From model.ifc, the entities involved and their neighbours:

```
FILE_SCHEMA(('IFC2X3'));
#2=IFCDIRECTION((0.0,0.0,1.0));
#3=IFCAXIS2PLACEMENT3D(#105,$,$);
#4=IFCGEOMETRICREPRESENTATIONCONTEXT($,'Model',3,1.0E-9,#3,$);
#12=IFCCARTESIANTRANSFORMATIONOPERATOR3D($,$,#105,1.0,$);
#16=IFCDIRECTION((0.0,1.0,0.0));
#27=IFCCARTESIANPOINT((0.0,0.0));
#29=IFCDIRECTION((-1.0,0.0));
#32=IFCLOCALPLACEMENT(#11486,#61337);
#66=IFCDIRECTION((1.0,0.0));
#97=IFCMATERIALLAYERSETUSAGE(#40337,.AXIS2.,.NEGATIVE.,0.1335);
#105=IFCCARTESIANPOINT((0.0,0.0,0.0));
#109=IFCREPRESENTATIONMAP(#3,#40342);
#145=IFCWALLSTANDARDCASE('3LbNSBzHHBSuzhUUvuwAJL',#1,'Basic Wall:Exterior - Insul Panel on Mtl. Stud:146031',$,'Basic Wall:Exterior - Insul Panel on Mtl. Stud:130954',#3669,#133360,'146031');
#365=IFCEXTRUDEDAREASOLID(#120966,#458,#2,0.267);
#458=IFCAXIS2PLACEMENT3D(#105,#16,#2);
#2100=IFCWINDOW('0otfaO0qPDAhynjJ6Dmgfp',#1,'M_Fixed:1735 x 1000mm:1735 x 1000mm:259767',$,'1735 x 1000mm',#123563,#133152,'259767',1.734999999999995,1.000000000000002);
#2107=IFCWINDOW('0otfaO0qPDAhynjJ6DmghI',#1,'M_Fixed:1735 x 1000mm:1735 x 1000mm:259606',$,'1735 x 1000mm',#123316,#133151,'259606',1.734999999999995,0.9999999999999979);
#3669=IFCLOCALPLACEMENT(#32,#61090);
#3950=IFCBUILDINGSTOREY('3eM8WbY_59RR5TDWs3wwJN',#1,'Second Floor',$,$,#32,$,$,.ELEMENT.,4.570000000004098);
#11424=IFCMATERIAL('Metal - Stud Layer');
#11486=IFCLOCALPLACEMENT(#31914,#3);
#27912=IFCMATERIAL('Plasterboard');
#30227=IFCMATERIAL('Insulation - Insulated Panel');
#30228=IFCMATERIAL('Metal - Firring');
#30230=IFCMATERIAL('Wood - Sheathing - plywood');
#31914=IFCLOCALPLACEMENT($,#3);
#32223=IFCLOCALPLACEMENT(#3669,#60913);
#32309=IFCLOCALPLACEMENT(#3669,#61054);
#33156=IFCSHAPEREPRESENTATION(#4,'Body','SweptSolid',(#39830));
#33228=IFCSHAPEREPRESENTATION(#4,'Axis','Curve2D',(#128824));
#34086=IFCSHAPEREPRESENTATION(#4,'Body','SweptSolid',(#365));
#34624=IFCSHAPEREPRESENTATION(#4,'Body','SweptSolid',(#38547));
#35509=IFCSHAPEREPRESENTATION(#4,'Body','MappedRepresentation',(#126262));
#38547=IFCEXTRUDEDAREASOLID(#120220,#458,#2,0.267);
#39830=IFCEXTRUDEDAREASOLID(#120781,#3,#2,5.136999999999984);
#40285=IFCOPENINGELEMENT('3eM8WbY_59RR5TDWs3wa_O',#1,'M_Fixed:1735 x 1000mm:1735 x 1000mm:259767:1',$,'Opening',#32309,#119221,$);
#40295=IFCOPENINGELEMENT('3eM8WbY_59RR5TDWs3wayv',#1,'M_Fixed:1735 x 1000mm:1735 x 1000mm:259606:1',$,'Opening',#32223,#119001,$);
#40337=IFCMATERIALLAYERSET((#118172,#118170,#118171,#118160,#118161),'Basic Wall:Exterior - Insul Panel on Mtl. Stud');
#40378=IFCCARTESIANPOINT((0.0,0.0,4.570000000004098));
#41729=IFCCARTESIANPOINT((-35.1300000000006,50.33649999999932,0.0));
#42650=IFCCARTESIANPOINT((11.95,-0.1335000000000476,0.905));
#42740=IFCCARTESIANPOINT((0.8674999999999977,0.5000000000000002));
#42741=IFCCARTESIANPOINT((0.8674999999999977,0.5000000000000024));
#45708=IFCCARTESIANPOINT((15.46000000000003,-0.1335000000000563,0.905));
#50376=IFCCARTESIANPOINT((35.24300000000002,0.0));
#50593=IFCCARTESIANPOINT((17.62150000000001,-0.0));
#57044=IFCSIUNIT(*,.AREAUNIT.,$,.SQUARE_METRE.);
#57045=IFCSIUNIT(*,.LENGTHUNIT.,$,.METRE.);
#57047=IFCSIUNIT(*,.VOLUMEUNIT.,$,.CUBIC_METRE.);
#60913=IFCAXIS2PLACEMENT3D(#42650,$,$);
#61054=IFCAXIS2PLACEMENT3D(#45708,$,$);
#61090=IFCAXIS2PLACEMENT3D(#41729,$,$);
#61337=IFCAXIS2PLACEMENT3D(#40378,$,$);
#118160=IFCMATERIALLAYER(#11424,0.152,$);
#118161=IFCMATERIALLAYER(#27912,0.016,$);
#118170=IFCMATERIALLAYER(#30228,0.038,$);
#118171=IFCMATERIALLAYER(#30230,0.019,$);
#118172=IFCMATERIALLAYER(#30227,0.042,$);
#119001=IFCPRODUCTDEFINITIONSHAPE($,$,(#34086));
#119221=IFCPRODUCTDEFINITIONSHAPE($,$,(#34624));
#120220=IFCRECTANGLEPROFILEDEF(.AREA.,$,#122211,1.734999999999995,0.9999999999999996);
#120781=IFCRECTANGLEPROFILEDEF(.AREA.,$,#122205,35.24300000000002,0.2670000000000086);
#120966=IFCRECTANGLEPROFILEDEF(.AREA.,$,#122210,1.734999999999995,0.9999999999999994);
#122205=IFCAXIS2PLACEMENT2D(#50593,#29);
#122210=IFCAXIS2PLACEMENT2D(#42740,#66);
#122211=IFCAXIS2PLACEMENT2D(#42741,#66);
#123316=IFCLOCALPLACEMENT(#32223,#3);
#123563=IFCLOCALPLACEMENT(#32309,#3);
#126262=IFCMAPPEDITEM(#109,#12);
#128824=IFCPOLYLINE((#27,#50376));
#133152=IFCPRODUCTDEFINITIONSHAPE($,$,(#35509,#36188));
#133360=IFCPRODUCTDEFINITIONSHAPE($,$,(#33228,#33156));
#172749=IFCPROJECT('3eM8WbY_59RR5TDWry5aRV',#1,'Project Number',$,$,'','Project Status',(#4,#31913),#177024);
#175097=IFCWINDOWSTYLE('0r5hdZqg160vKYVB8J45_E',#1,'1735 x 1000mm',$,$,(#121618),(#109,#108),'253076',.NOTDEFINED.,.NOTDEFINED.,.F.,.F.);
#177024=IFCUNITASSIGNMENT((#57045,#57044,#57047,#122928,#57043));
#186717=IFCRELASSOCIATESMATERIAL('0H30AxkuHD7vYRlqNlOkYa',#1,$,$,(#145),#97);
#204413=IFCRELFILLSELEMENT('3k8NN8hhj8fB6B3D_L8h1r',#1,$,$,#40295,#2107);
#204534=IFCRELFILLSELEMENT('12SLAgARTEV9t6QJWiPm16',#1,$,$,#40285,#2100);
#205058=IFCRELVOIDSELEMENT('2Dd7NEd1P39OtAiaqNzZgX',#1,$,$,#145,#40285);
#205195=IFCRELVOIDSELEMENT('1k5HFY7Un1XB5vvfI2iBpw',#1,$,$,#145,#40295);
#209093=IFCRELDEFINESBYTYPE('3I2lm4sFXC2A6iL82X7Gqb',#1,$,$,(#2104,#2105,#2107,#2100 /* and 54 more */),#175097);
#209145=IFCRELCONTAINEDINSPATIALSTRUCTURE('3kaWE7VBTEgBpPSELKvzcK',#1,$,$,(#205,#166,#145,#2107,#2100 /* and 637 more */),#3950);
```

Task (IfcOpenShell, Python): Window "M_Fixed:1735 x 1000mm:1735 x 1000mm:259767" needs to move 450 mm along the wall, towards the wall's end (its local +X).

```python
import ifcopenshell
import ifcopenshell.api.geometry
import ifcopenshell.util.placement
import ifcopenshell.util.unit

model = ifcopenshell.open("model.ifc")
unit_scale = ifcopenshell.util.unit.calculate_unit_scale(model)

window = model.by_id(2100)
opening = window.FillsVoids[0].RelatingOpeningElement
wall = opening.VoidsElements[0].RelatingBuildingElement

wall_matrix = ifcopenshell.util.placement.get_local_placement(wall.ObjectPlacement)
shift = wall_matrix[:3, 0] * 0.45 / unit_scale
before = ifcopenshell.util.placement.get_local_placement(window.ObjectPlacement)[:3, 3].copy()

# The window is placed relative to its opening, so it follows when the opening moves.
matrix = ifcopenshell.util.placement.get_local_placement(opening.ObjectPlacement)
matrix[:3, 3] += shift
ifcopenshell.api.geometry.edit_object_placement(
    model, product=opening, matrix=matrix, is_si=False, should_transform_children=True
)

after = ifcopenshell.util.placement.get_local_placement(window.ObjectPlacement)[:3, 3]
print("window moved by", (after - before).round(3) + 0.0)

model.write("model_edited.ifc")
```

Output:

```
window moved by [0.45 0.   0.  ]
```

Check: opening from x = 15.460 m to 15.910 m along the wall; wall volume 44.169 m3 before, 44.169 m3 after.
